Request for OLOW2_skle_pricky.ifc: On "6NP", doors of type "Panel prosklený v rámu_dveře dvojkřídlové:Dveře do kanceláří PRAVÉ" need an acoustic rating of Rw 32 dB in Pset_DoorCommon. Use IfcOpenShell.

First a look at what the model holds.

```python
import ifcopenshell
import ifcopenshell.util.element

model = ifcopenshell.open("OLOW2_skle_pricky.ifc")
print(model.schema)
storey = next(s for s in model.by_type("IfcBuildingStorey") if s.Name == "6NP")
doors = [e for e in ifcopenshell.util.element.get_decomposition(storey) if e.is_a("IfcDoor")]
seen = {}
for e in doors:
    element_type = ifcopenshell.util.element.get_type(e)
    key = (element_type.Name if element_type != e and element_type else None, ifcopenshell.util.element.get_pset(e, "Pset_DoorCommon", "AcousticRating"))
    seen[key] = seen.get(key, 0) + 1
for (name, value), count in sorted(seen.items(), key=str):
    print(count, "x", name, "|", value)
```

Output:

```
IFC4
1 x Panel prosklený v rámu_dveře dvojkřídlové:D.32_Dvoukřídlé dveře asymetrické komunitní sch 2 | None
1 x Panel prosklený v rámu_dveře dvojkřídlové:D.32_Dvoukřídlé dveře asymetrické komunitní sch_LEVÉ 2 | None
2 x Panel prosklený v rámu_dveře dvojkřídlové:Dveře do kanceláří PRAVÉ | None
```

```python
import ifcopenshell
import ifcopenshell.api.pset
import ifcopenshell.util.element

model = ifcopenshell.open("OLOW2_skle_pricky.ifc")

storey = next(s for s in model.by_type("IfcBuildingStorey") if s.Name == "6NP")
doors = [e for e in ifcopenshell.util.element.get_decomposition(storey) if e.is_a("IfcDoor")]

count = 0
for e in doors:
    element_type = ifcopenshell.util.element.get_type(e)
    if element_type in (None, e) or element_type.Name != "Panel prosklený v rámu_dveře dvojkřídlové:Dveře do kanceláří PRAVÉ":
        continue
    # add_pset returns the element's existing set when there is one.
    pset = ifcopenshell.api.pset.add_pset(model, product=e, name="Pset_DoorCommon")
    ifcopenshell.api.pset.edit_pset(model, pset=pset, properties={"AcousticRating": "Rw 32 dB"})
    count += 1

print(count, "doors updated")

model.write("OLOW2_skle_pricky_v2.ifc")
```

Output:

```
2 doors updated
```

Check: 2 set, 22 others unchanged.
